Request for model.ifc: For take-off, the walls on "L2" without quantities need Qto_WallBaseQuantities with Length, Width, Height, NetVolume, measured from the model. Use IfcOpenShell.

First a look at what the model holds.

```python
import ifcopenshell
import ifcopenshell.util.element
import ifcopenshell.util.unit

model = ifcopenshell.open("model.ifc")
print(model.schema)
for unit_type in ("LENGTHUNIT", "AREAUNIT", "VOLUMEUNIT"):
    print(unit_type, ifcopenshell.util.unit.calculate_unit_scale(model, unit_type))
storey = next(s for s in model.by_type("IfcBuildingStorey") if s.Name == "L2")
walls = [e for e in ifcopenshell.util.element.get_decomposition(storey) if e.is_a("IfcWall")]
for e in sorted(walls, key=lambda e: e.id()):
    print(e.id(), e.is_a(), e.Name, list(ifcopenshell.util.element.get_psets(e, qtos_only=True)), sep=" | ")
```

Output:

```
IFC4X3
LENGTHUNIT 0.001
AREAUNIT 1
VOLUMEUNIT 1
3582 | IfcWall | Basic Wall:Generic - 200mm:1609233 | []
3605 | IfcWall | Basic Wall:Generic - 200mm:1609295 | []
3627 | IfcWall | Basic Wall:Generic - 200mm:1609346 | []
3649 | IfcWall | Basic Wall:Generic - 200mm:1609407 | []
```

```python
import ifcopenshell
import ifcopenshell.api.pset
import ifcopenshell.geom
import ifcopenshell.util.element
import ifcopenshell.util.shape
import ifcopenshell.util.unit

model = ifcopenshell.open("model.ifc")
unit_scale = ifcopenshell.util.unit.calculate_unit_scale(model)
volume_scale = ifcopenshell.util.unit.calculate_unit_scale(model, "VOLUMEUNIT")
settings = ifcopenshell.geom.settings()

storey = next(s for s in model.by_type("IfcBuildingStorey") if s.Name == "L2")
walls = [e for e in ifcopenshell.util.element.get_decomposition(storey) if e.is_a("IfcWall")]

for e in sorted(walls, key=lambda e: e.id()):
    if ifcopenshell.util.element.get_psets(e, qtos_only=True, should_inherit=False):
        continue
    # Geometry comes back in metres, in the element's own axes.
    shape = ifcopenshell.geom.create_shape(settings, e)
    values = {
        "Length": ifcopenshell.util.shape.get_x(shape.geometry) / unit_scale,
        "Width": ifcopenshell.util.shape.get_y(shape.geometry) / unit_scale,
        "Height": ifcopenshell.util.shape.get_z(shape.geometry) / unit_scale,
        "NetVolume": ifcopenshell.util.shape.get_volume(shape.geometry) / volume_scale,
    }
    qto = ifcopenshell.api.pset.add_qto(model, product=e, name="Qto_WallBaseQuantities")
    ifcopenshell.api.pset.edit_qto(model, qto=qto, properties=values)
    print(e.id(), {k: round(v, 3) for k, v in values.items()})

model.write("model_rev.ifc")
```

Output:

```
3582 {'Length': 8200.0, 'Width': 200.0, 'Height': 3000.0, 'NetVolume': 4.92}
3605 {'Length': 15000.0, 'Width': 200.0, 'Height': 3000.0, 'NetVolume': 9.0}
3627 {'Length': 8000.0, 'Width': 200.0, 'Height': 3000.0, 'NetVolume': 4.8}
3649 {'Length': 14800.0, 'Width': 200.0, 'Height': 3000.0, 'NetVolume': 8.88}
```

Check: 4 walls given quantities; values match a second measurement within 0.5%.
